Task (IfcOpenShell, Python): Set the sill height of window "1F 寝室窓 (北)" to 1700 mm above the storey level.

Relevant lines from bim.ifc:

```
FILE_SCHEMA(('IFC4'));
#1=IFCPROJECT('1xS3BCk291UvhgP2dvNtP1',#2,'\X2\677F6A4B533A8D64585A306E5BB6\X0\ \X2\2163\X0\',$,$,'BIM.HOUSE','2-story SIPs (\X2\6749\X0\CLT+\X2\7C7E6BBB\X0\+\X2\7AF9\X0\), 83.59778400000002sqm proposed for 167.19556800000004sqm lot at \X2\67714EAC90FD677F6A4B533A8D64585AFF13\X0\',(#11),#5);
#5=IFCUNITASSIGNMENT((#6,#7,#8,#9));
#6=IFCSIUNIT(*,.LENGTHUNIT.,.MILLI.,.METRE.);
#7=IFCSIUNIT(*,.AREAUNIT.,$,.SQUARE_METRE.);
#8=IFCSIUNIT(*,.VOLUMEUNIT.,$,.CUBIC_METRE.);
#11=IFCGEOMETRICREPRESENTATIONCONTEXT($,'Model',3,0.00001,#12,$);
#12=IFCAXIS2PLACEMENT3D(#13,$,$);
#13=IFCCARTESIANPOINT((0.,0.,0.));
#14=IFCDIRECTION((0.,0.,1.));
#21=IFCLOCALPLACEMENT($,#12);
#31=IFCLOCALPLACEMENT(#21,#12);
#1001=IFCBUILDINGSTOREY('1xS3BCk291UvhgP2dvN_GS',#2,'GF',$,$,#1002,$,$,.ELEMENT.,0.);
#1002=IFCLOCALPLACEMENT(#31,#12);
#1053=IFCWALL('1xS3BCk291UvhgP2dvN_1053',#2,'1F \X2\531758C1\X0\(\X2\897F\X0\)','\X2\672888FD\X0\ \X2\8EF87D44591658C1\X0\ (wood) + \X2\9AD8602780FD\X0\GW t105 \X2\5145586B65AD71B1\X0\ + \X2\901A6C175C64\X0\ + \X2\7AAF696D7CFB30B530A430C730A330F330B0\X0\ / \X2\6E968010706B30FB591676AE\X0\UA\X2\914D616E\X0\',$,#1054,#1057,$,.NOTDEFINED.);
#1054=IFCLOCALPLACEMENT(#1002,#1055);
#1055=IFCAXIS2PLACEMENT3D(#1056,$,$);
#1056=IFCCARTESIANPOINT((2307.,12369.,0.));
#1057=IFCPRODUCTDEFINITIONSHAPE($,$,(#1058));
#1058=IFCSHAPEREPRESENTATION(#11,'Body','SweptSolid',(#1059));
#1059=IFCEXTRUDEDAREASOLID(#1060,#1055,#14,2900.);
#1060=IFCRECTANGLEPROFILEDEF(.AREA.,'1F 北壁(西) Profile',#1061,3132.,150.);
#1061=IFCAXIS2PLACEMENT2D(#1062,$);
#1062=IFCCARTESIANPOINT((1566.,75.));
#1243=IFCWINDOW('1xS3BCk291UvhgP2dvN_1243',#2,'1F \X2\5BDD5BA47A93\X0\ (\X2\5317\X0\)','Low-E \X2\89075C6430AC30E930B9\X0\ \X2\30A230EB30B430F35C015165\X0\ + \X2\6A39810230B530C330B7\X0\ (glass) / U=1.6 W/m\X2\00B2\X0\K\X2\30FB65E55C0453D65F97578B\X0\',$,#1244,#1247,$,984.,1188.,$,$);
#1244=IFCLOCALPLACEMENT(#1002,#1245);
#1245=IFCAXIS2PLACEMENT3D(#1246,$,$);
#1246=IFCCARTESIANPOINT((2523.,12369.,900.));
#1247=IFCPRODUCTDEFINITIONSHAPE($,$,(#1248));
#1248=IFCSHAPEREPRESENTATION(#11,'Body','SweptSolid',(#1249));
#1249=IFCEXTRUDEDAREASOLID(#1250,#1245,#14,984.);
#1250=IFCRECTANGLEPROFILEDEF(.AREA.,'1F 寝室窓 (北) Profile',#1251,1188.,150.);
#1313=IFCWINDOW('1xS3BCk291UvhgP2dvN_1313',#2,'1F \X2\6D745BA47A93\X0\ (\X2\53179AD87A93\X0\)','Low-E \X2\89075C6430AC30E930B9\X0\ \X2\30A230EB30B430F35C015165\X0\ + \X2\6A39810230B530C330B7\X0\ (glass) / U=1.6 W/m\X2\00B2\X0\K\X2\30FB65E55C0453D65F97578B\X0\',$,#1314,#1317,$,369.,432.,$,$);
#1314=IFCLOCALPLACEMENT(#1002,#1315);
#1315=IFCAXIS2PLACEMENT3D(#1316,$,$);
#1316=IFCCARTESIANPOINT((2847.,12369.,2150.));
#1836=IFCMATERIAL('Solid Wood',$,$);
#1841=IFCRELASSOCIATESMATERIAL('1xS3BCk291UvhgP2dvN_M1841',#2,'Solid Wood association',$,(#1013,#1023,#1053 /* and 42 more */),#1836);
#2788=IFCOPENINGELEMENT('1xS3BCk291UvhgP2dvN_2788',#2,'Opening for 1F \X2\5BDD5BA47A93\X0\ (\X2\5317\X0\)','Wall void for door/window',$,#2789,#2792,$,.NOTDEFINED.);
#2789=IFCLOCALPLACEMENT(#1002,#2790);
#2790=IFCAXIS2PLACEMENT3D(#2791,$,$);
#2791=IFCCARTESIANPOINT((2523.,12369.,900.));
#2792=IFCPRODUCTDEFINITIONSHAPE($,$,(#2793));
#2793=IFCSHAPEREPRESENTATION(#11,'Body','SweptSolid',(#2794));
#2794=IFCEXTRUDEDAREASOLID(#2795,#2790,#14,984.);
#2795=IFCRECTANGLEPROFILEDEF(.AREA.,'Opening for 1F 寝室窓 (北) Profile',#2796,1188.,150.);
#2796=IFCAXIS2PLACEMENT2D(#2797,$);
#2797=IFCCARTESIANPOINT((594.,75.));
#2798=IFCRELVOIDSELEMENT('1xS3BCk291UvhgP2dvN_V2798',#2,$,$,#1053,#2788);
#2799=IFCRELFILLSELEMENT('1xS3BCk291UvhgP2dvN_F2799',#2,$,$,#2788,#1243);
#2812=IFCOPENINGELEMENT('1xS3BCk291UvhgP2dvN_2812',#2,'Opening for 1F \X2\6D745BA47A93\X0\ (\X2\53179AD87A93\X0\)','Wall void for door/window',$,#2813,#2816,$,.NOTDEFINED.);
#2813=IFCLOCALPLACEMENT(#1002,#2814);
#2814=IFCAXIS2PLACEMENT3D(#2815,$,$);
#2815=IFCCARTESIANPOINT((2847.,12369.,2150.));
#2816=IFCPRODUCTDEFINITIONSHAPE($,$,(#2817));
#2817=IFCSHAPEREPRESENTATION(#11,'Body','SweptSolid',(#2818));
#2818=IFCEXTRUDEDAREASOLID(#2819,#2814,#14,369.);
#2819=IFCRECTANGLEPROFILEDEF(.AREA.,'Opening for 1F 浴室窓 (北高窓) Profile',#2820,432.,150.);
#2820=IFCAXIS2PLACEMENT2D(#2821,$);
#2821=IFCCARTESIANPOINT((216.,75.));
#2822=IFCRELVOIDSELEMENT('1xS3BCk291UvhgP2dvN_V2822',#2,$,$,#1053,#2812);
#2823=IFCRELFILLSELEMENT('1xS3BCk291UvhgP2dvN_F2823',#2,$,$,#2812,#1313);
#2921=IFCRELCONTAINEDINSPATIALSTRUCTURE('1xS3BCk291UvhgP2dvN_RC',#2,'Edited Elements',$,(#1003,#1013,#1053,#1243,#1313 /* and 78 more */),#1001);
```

```python
import numpy as np
import ifcopenshell
import ifcopenshell.api.geometry
import ifcopenshell.geom
import ifcopenshell.util.element
import ifcopenshell.util.placement
import ifcopenshell.util.shape
import ifcopenshell.util.unit

model = ifcopenshell.open("bim.ifc")
unit_scale = ifcopenshell.util.unit.calculate_unit_scale(model)

window = model.by_guid("1xS3BCk291UvhgP2dvN_1243")
opening = window.FillsVoids[0].RelatingOpeningElement
storey = ifcopenshell.util.element.get_container(window, ifc_class="IfcBuildingStorey")
level = ifcopenshell.util.placement.get_local_placement(storey.ObjectPlacement)[2, 3]

# The opening's origin need not be at the sill, so measure its lowest point.
shape = ifcopenshell.geom.create_shape(ifcopenshell.geom.settings(), opening)
bottom = ifcopenshell.util.shape.get_shape_bottom_elevation(shape, shape.geometry) / unit_scale
dz = level + 1.7 / unit_scale - bottom

shift = np.array([0.0, 0.0, dz])
# The window is not placed relative to its opening, so move both.
for product in (opening, window):
    matrix = ifcopenshell.util.placement.get_local_placement(product.ObjectPlacement)
    matrix[:3, 3] += shift
    ifcopenshell.api.geometry.edit_object_placement(model, product=product, matrix=matrix, is_si=False)

print(f"moved by {dz * unit_scale:+.3f} m")

model.write("bim-out.ifc")
```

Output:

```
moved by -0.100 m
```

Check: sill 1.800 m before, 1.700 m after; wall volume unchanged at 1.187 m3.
